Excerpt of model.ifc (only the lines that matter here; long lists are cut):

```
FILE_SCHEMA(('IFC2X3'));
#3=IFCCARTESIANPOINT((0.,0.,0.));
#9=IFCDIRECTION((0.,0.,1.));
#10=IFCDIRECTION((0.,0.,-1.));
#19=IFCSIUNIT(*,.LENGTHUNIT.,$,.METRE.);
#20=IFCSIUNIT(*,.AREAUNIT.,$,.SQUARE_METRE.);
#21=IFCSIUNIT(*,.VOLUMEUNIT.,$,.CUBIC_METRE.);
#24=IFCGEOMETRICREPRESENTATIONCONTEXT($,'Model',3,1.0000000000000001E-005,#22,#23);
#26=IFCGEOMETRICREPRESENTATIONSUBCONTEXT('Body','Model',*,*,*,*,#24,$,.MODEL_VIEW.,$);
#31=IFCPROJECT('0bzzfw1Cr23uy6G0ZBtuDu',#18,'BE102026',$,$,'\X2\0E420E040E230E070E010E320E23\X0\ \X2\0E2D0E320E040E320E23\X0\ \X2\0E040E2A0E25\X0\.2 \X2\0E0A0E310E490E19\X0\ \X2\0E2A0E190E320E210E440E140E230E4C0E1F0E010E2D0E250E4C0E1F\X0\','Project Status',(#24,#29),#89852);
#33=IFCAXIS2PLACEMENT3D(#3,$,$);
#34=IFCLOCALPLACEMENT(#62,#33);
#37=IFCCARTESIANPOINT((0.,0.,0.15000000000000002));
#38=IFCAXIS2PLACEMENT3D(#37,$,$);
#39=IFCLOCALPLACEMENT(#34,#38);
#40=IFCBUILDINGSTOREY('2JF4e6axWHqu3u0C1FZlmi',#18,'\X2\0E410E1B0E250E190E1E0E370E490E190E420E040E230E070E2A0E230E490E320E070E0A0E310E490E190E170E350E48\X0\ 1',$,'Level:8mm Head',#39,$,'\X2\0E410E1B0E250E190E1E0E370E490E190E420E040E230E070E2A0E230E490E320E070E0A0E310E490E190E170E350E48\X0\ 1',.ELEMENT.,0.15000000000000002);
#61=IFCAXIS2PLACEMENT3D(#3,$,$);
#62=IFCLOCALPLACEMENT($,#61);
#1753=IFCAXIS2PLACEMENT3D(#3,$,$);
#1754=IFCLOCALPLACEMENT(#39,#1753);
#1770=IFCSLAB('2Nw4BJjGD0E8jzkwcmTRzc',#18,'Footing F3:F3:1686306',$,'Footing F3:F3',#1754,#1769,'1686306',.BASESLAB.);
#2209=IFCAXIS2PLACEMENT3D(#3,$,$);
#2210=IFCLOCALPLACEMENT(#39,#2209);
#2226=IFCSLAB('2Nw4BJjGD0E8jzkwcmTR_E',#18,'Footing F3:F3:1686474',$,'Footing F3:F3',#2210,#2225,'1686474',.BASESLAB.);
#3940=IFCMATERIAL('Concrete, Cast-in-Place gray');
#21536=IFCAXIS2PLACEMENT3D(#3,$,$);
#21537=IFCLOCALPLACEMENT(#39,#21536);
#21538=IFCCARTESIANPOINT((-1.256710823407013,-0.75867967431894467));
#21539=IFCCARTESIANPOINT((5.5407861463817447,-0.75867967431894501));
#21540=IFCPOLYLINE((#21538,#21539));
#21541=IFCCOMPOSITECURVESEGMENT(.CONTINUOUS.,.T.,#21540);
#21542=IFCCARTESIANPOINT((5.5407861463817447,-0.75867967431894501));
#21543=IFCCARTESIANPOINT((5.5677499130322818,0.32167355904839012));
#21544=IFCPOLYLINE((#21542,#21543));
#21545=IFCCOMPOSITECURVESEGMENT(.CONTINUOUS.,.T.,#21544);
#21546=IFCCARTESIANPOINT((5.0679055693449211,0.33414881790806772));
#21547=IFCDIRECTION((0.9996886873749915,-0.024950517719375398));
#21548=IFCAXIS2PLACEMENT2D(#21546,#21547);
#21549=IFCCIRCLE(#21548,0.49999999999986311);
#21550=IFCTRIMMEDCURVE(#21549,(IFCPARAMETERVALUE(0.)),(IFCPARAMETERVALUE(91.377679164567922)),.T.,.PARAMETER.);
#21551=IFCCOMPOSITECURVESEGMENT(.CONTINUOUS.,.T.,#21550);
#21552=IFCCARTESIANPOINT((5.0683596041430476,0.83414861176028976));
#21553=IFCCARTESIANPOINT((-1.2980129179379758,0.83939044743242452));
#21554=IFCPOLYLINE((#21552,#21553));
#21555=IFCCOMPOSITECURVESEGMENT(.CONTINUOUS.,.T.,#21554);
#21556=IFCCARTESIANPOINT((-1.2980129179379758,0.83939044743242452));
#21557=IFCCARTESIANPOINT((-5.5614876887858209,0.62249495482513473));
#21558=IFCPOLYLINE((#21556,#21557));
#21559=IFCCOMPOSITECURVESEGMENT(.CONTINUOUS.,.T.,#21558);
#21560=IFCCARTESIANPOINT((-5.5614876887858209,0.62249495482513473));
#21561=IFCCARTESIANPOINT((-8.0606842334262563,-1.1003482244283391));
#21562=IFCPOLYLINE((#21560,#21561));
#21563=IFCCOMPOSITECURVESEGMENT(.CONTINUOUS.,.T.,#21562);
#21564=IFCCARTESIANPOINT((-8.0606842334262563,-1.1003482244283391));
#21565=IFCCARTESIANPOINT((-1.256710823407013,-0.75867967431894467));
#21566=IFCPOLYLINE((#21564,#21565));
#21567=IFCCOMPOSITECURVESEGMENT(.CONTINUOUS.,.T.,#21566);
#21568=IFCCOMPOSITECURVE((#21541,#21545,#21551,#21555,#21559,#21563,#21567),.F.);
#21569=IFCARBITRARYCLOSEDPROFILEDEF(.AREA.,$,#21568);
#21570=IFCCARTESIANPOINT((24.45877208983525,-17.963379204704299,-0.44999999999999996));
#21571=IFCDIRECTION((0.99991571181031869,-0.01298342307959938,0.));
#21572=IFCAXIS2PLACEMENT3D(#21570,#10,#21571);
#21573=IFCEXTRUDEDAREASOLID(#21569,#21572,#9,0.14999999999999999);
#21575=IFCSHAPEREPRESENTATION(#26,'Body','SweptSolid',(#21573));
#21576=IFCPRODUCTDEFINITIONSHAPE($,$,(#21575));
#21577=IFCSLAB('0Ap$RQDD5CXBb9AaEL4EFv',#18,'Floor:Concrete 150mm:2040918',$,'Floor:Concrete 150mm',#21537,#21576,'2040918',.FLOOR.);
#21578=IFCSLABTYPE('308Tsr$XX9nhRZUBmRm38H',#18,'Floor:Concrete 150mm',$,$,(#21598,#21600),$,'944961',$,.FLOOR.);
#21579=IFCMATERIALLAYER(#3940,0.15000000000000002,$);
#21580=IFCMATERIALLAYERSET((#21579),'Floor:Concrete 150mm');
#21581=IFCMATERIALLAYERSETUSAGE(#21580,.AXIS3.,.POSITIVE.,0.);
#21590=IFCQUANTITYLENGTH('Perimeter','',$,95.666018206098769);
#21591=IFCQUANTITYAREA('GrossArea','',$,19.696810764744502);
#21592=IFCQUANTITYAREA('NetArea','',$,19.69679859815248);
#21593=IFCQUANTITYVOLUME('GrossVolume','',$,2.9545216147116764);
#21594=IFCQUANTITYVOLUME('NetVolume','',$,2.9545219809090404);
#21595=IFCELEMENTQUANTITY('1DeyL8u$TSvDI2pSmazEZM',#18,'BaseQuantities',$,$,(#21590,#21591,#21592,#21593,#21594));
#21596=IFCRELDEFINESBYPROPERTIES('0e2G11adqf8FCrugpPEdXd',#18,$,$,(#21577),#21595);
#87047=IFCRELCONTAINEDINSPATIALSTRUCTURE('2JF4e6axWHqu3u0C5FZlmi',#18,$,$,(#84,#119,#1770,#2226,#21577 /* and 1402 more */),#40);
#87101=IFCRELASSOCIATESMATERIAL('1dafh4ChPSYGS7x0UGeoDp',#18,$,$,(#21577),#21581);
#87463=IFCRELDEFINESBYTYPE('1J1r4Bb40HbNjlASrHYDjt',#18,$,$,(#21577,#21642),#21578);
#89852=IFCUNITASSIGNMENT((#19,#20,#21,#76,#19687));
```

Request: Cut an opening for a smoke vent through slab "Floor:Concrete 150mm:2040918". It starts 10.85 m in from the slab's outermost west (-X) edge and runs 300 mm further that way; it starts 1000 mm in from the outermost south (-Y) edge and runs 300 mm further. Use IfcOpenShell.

```python
import numpy as np
import ifcopenshell
import ifcopenshell.api.feature
import ifcopenshell.api.geometry
import ifcopenshell.api.pset
import ifcopenshell.api.root
import ifcopenshell.geom
import ifcopenshell.util.element
import ifcopenshell.util.placement
import ifcopenshell.util.representation
import ifcopenshell.util.shape
import ifcopenshell.util.unit

model = ifcopenshell.open("model.ifc")
unit_scale = ifcopenshell.util.unit.calculate_unit_scale(model)
area_scale = ifcopenshell.util.unit.calculate_unit_scale(model, "AREAUNIT")
volume_scale = ifcopenshell.util.unit.calculate_unit_scale(model, "VOLUMEUNIT")
settings = ifcopenshell.geom.settings()


def volume(element):
    """Net volume in cubic metres, openings subtracted."""
    shape = ifcopenshell.geom.create_shape(settings, element)
    return ifcopenshell.util.shape.get_volume(shape.geometry)


slab = model.by_guid("0Ap$RQDD5CXBb9AaEL4EFv")
before = volume(slab)

# Extent in the slab's own axes, in metres. The edges named are its -X and -Y sides.
slab_shape = ifcopenshell.geom.create_shape(settings, slab)
vertices = ifcopenshell.util.shape.get_vertices(slab_shape.geometry)
x_min, y_min, bottom = vertices.min(axis=0)
top = vertices[:, 2].max()

opening = ifcopenshell.api.root.create_entity(model, ifc_class="IfcOpeningElement", name="Smoke vent opening")
context = ifcopenshell.util.representation.get_context(model, "Model", "Body", "MODEL_VIEW")
width, depth = 0.3, 0.3
outline = [(0.0, 0.0), (width, 0.0), (width, depth), (0.0, depth), (0.0, 0.0)]
# Overshoot both faces by 50 mm so the cut is clean.
shape = ifcopenshell.api.geometry.add_slab_representation(
    model, context=context, depth=top - bottom + 0.1, polyline=outline
)
ifcopenshell.api.geometry.assign_representation(model, product=opening, representation=shape)

matrix = ifcopenshell.util.placement.get_local_placement(slab.ObjectPlacement)
matrix[:, 3] = matrix @ np.append(np.array([x_min + 10.85, y_min + 1, bottom - 0.05]) / unit_scale, 1.0)
ifcopenshell.api.geometry.edit_object_placement(model, product=opening, matrix=matrix, is_si=False)
ifcopenshell.api.feature.add_feature(model, feature=opening, element=slab)

after = volume(slab)

# Update the slab's stored quantities.
qto = model.by_id(ifcopenshell.util.element.get_pset(slab, "BaseQuantities", should_inherit=False)["id"])
ifcopenshell.api.pset.edit_qto(model, qto=qto, properties={
    "NetArea": after / (top - bottom) / area_scale,
    "NetVolume": after / volume_scale,
})

print(f"slab volume {before:.3f} -> {after:.3f} m3")

model.write("model_updated.ifc")
```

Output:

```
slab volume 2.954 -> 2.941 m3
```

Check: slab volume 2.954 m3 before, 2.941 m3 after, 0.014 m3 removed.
